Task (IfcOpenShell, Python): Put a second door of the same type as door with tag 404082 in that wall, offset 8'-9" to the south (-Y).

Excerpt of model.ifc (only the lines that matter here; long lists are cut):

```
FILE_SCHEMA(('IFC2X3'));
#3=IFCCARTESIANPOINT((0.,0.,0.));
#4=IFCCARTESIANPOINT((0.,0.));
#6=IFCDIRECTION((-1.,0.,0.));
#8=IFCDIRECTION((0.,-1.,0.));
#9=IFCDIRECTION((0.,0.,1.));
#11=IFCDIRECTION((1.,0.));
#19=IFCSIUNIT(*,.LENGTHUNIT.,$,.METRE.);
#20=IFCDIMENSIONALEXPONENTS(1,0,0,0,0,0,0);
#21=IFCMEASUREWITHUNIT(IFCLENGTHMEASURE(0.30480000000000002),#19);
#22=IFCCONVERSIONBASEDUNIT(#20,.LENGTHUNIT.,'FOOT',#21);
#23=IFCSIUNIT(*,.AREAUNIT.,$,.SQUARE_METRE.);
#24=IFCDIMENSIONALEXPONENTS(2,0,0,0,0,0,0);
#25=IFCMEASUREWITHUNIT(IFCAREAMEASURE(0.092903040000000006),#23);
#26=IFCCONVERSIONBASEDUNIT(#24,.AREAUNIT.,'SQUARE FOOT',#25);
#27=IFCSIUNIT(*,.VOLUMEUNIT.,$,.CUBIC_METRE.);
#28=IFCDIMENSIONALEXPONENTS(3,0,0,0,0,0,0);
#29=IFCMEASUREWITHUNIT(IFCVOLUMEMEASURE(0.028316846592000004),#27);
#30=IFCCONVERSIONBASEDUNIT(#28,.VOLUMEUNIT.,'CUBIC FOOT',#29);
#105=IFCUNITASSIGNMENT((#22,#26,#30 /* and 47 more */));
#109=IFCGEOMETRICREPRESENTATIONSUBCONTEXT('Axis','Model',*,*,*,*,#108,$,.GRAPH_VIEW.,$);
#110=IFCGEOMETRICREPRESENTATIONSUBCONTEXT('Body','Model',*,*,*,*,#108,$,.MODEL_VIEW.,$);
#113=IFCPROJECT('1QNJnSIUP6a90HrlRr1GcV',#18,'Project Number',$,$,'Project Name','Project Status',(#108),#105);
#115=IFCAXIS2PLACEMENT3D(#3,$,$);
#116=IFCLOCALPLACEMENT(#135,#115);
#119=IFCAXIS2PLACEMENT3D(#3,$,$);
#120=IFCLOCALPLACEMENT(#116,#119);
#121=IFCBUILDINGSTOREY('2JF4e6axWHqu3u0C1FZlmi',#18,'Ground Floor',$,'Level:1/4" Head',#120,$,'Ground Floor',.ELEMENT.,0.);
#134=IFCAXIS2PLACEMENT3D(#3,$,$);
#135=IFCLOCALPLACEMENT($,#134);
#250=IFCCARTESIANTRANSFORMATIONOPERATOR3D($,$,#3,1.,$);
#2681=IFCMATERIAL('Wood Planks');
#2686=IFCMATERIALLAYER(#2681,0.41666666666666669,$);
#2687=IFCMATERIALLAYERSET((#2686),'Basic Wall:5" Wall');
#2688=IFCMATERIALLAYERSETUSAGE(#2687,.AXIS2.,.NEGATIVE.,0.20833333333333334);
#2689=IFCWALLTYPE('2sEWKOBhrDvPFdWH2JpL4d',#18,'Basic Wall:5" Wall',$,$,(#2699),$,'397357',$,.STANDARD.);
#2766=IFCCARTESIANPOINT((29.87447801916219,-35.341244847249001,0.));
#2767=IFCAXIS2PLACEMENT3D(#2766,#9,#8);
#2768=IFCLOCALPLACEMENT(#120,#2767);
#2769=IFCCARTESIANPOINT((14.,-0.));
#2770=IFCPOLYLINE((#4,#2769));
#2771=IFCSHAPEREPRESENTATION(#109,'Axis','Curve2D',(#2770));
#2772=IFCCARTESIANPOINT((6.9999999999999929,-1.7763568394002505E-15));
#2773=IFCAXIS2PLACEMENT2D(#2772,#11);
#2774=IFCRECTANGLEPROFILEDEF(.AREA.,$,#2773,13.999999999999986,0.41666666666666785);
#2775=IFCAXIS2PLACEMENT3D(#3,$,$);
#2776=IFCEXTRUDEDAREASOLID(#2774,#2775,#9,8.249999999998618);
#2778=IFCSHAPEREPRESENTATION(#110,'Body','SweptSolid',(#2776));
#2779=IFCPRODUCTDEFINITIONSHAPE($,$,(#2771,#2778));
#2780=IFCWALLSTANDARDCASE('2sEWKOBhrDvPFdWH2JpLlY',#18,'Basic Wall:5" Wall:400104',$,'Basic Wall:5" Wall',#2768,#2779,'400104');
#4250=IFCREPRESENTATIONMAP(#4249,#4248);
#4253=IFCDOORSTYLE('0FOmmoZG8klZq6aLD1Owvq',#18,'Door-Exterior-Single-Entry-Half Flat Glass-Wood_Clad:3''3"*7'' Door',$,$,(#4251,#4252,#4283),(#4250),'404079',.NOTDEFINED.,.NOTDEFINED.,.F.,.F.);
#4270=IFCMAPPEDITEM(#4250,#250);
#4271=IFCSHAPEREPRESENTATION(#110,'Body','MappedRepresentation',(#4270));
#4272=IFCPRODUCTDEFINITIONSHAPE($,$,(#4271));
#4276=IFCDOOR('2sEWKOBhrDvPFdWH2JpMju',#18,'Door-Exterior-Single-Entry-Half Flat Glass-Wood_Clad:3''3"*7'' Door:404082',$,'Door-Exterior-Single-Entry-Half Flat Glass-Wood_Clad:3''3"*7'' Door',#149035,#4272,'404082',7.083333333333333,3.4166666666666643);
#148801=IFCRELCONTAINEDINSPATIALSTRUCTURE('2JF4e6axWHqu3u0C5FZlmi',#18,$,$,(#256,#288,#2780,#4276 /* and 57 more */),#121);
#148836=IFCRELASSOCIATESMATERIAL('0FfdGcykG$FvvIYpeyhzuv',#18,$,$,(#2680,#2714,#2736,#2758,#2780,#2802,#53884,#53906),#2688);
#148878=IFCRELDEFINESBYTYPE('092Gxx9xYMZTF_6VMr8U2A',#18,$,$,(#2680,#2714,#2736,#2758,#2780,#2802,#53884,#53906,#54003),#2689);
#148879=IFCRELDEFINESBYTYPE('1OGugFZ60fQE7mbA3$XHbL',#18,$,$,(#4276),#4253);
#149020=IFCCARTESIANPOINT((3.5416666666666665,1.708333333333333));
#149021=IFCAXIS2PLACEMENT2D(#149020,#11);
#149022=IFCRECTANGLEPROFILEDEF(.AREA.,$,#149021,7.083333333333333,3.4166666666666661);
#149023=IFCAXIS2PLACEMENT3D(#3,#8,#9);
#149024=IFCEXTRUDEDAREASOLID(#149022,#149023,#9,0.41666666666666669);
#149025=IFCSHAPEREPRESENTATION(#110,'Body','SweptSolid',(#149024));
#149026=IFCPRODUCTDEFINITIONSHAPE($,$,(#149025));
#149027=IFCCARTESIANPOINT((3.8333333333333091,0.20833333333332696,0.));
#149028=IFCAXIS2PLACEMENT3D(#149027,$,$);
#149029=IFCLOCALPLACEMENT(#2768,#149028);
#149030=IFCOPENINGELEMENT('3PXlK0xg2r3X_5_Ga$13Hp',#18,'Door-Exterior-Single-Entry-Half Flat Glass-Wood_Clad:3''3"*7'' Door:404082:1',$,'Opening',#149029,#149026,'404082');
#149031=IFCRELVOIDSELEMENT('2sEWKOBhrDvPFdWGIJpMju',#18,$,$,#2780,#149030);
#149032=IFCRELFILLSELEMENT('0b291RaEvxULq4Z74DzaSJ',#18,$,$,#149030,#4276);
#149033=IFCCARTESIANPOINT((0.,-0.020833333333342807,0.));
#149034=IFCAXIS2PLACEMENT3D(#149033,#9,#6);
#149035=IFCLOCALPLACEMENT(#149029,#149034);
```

```python
import ifcopenshell
import ifcopenshell.api.feature
import ifcopenshell.api.geometry
import ifcopenshell.api.root
import ifcopenshell.geom
import ifcopenshell.util.element
import ifcopenshell.util.placement
import ifcopenshell.util.shape
import ifcopenshell.util.unit

model = ifcopenshell.open("model.ifc")
unit_scale = ifcopenshell.util.unit.calculate_unit_scale(model)
settings = ifcopenshell.geom.settings()


def volume(element):
    """Net volume in cubic metres, openings subtracted."""
    shape = ifcopenshell.geom.create_shape(settings, element)
    return ifcopenshell.util.shape.get_volume(shape.geometry)


def reuse_history(source, copy):
    """copy_class also copies each property set's owner history, people and application; keep the originals."""
    for rel in copy.IsDefinedBy:
        if rel.is_a("IfcRelDefinesByProperties") and (history := rel.RelatingPropertyDefinition.OwnerHistory):
            rel.RelatingPropertyDefinition.OwnerHistory = source.OwnerHistory
            ifcopenshell.util.element.remove_deep2(model, history)


door = model.by_guid("2sEWKOBhrDvPFdWH2JpMju")
opening = door.FillsVoids[0].RelatingOpeningElement
wall = opening.VoidsElements[0].RelatingBuildingElement
before = volume(wall)
shift = ifcopenshell.util.placement.get_local_placement(wall.ObjectPlacement)[:3, 0] * 105 * 0.0254 / unit_scale

# copy_class copies the void relationship, type, container and properties, but no geometry.
new_opening = ifcopenshell.api.root.copy_class(model, product=opening)
new_opening.Representation = ifcopenshell.util.element.copy_deep(
    model, opening.Representation, exclude=["IfcGeometricRepresentationContext", "IfcRepresentationMap"]
)
new_opening.Name = 'Door-Exterior-Single-Entry-Half Flat Glass-Wood_Clad:3\'3"*7\' Door'
new_opening.Tag = None
new_door = ifcopenshell.api.root.copy_class(model, product=door)
new_door.Representation = ifcopenshell.util.element.copy_deep(
    model, door.Representation, exclude=["IfcGeometricRepresentationContext", "IfcRepresentationMap"]
)
new_door.Name = 'Door-Exterior-Single-Entry-Half Flat Glass-Wood_Clad:3\'3"*7\' Door'
new_door.Tag = None
reuse_history(door, new_door)
fills = ifcopenshell.api.feature.add_filling(model, opening=new_opening, element=new_door)
fills.OwnerHistory = new_door.OwnerHistory  # required in IFC2X3

for old, new in ((opening, new_opening), (door, new_door)):
    matrix = ifcopenshell.util.placement.get_local_placement(old.ObjectPlacement)
    matrix[:3, 3] += shift
    ifcopenshell.api.geometry.edit_object_placement(model, product=new, matrix=matrix, is_si=False)

after = volume(wall)

print(f"wall volume {before:.3f} -> {after:.3f} m3")

model.write("model_edited.ifc")
```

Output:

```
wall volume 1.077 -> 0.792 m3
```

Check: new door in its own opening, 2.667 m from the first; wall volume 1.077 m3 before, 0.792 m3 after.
